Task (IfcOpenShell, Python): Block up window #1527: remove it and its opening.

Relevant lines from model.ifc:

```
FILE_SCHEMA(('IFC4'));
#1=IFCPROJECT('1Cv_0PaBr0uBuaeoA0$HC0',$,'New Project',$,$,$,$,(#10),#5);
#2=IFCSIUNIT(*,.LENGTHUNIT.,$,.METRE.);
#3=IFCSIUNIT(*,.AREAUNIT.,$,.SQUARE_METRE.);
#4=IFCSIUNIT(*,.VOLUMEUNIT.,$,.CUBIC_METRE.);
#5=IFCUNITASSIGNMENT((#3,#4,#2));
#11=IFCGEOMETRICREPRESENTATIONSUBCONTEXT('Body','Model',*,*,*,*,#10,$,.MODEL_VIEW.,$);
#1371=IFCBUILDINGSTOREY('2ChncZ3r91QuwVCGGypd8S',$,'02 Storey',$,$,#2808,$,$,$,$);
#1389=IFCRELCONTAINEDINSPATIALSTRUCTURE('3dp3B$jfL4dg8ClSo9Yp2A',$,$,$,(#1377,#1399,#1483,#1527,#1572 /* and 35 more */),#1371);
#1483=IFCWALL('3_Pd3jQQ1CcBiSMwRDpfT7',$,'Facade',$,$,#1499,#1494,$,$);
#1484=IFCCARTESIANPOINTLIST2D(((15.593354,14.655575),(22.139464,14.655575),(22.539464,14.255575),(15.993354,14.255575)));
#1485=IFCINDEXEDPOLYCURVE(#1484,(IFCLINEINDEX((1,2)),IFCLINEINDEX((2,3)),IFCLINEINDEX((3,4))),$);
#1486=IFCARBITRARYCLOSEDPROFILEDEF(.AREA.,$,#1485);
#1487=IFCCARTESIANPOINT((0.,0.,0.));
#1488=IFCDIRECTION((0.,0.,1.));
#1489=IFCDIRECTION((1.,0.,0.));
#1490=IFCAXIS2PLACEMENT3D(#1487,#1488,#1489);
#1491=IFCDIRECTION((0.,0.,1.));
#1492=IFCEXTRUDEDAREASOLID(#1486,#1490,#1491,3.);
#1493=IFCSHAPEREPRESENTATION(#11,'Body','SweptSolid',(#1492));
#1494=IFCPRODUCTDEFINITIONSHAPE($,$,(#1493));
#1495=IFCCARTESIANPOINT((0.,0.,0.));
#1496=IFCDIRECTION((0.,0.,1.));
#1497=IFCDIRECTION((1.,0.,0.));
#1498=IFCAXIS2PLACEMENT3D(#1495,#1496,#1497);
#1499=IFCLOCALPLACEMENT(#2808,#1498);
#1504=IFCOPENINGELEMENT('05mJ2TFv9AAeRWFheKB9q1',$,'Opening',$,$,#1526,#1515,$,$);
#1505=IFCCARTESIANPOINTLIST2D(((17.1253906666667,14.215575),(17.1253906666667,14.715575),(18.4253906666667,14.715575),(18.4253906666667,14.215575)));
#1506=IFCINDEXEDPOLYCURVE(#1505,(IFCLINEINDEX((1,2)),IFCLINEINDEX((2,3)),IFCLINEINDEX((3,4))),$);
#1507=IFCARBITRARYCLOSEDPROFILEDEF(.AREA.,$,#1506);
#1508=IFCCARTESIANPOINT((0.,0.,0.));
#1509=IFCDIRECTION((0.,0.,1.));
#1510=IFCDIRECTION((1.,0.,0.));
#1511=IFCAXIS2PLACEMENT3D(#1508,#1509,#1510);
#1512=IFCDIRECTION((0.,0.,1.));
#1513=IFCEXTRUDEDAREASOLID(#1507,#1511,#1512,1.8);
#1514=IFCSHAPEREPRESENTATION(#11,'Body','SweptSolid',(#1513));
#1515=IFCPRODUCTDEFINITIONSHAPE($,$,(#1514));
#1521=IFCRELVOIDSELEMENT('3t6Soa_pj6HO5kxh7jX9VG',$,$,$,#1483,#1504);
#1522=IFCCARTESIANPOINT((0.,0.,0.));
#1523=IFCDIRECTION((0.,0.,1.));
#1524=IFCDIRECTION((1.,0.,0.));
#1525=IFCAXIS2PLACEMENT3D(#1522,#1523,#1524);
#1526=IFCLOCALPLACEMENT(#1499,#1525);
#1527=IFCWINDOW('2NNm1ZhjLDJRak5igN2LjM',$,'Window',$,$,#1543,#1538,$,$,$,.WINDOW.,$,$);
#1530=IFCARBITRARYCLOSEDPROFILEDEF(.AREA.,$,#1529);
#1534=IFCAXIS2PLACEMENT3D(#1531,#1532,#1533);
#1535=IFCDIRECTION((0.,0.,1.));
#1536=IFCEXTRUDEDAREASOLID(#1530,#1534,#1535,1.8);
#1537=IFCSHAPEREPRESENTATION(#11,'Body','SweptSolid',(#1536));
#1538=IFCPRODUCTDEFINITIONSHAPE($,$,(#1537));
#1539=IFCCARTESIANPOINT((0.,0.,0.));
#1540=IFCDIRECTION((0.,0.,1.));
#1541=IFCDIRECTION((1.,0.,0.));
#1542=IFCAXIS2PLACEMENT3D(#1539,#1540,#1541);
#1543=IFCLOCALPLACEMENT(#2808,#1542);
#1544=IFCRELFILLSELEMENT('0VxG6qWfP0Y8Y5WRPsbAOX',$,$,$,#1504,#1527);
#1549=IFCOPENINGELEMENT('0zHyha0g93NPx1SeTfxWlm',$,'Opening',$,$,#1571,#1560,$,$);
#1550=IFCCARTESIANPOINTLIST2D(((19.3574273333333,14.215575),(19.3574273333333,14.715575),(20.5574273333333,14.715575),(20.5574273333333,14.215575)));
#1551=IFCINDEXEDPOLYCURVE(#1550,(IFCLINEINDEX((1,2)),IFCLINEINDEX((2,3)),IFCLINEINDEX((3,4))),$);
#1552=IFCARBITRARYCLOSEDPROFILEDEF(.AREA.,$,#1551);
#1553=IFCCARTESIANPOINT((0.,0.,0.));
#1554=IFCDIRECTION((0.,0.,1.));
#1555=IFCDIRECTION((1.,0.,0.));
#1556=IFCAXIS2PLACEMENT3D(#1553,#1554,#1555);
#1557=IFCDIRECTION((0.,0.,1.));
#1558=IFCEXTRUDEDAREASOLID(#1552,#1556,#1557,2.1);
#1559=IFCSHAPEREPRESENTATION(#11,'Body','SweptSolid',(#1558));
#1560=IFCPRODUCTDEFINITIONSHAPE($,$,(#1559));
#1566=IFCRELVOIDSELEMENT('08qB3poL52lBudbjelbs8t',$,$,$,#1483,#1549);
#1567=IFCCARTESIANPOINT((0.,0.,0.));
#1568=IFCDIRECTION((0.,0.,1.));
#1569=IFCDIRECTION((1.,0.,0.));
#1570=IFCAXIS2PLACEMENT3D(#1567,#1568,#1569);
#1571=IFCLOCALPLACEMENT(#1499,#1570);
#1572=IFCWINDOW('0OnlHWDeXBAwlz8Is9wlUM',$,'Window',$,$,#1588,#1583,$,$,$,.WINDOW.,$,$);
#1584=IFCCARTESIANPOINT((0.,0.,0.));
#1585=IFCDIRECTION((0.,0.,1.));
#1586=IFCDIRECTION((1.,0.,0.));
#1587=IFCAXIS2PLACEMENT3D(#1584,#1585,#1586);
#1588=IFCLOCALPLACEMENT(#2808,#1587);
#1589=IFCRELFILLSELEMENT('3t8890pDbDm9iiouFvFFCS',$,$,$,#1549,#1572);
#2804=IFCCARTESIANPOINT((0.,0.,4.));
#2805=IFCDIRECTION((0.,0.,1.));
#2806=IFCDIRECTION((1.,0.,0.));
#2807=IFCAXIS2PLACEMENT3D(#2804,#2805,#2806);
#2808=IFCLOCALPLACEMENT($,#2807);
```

```python
import ifcopenshell
import ifcopenshell.api.feature
import ifcopenshell.api.root
import ifcopenshell.geom
import ifcopenshell.util.shape

model = ifcopenshell.open("model.ifc")
settings = ifcopenshell.geom.settings()


def volume(element):
    """Net volume in cubic metres, openings subtracted."""
    shape = ifcopenshell.geom.create_shape(settings, element)
    return ifcopenshell.util.shape.get_volume(shape.geometry)


window = model.by_guid("2NNm1ZhjLDJRak5igN2LjM")
opening = window.FillsVoids[0].RelatingOpeningElement
wall = opening.VoidsElements[0].RelatingBuildingElement
before = volume(wall)

ifcopenshell.api.root.remove_product(model, product=window)
ifcopenshell.api.feature.remove_feature(model, feature=opening)

after = volume(wall)

print(f"wall volume {before:.3f} -> {after:.3f} m3")

model.write("model_rev.ifc")
```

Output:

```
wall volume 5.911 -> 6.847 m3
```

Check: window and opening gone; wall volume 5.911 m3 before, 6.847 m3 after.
